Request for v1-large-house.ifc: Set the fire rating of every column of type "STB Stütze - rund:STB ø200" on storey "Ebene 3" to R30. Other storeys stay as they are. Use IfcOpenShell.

First a look at what the model holds.

```python
import ifcopenshell
import ifcopenshell.util.element

model = ifcopenshell.open("v1-large-house.ifc")
print(model.schema)
storey = next(s for s in model.by_type("IfcBuildingStorey") if s.Name == "Ebene 3")
columns = [e for e in ifcopenshell.util.element.get_decomposition(storey) if e.is_a("IfcColumn")]
seen = {}
for e in columns:
    element_type = ifcopenshell.util.element.get_type(e)
    key = (element_type.Name if element_type != e and element_type else None, ifcopenshell.util.element.get_pset(e, "Pset_ColumnCommon", "FireRating"))
    seen[key] = seen.get(key, 0) + 1
for (name, value), count in sorted(seen.items(), key=str):
    print(count, "x", name, "|", value)
```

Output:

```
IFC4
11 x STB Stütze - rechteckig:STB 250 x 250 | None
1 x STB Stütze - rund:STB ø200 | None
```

```python
import ifcopenshell
import ifcopenshell.api.pset
import ifcopenshell.util.element

model = ifcopenshell.open("v1-large-house.ifc")

storey = next(s for s in model.by_type("IfcBuildingStorey") if s.Name == "Ebene 3")
columns = [e for e in ifcopenshell.util.element.get_decomposition(storey) if e.is_a("IfcColumn")]

count = 0
for e in columns:
    element_type = ifcopenshell.util.element.get_type(e)
    if element_type in (None, e) or element_type.Name != "STB Stütze - rund:STB ø200":
        continue
    # add_pset returns the element's existing set when there is one.
    pset = ifcopenshell.api.pset.add_pset(model, product=e, name="Pset_ColumnCommon")
    ifcopenshell.api.pset.edit_pset(model, pset=pset, properties={"FireRating": "R30"})
    count += 1

print(count, "columns updated")

model.write("v1-large-house_edited.ifc")
```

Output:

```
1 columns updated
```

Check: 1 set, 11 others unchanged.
